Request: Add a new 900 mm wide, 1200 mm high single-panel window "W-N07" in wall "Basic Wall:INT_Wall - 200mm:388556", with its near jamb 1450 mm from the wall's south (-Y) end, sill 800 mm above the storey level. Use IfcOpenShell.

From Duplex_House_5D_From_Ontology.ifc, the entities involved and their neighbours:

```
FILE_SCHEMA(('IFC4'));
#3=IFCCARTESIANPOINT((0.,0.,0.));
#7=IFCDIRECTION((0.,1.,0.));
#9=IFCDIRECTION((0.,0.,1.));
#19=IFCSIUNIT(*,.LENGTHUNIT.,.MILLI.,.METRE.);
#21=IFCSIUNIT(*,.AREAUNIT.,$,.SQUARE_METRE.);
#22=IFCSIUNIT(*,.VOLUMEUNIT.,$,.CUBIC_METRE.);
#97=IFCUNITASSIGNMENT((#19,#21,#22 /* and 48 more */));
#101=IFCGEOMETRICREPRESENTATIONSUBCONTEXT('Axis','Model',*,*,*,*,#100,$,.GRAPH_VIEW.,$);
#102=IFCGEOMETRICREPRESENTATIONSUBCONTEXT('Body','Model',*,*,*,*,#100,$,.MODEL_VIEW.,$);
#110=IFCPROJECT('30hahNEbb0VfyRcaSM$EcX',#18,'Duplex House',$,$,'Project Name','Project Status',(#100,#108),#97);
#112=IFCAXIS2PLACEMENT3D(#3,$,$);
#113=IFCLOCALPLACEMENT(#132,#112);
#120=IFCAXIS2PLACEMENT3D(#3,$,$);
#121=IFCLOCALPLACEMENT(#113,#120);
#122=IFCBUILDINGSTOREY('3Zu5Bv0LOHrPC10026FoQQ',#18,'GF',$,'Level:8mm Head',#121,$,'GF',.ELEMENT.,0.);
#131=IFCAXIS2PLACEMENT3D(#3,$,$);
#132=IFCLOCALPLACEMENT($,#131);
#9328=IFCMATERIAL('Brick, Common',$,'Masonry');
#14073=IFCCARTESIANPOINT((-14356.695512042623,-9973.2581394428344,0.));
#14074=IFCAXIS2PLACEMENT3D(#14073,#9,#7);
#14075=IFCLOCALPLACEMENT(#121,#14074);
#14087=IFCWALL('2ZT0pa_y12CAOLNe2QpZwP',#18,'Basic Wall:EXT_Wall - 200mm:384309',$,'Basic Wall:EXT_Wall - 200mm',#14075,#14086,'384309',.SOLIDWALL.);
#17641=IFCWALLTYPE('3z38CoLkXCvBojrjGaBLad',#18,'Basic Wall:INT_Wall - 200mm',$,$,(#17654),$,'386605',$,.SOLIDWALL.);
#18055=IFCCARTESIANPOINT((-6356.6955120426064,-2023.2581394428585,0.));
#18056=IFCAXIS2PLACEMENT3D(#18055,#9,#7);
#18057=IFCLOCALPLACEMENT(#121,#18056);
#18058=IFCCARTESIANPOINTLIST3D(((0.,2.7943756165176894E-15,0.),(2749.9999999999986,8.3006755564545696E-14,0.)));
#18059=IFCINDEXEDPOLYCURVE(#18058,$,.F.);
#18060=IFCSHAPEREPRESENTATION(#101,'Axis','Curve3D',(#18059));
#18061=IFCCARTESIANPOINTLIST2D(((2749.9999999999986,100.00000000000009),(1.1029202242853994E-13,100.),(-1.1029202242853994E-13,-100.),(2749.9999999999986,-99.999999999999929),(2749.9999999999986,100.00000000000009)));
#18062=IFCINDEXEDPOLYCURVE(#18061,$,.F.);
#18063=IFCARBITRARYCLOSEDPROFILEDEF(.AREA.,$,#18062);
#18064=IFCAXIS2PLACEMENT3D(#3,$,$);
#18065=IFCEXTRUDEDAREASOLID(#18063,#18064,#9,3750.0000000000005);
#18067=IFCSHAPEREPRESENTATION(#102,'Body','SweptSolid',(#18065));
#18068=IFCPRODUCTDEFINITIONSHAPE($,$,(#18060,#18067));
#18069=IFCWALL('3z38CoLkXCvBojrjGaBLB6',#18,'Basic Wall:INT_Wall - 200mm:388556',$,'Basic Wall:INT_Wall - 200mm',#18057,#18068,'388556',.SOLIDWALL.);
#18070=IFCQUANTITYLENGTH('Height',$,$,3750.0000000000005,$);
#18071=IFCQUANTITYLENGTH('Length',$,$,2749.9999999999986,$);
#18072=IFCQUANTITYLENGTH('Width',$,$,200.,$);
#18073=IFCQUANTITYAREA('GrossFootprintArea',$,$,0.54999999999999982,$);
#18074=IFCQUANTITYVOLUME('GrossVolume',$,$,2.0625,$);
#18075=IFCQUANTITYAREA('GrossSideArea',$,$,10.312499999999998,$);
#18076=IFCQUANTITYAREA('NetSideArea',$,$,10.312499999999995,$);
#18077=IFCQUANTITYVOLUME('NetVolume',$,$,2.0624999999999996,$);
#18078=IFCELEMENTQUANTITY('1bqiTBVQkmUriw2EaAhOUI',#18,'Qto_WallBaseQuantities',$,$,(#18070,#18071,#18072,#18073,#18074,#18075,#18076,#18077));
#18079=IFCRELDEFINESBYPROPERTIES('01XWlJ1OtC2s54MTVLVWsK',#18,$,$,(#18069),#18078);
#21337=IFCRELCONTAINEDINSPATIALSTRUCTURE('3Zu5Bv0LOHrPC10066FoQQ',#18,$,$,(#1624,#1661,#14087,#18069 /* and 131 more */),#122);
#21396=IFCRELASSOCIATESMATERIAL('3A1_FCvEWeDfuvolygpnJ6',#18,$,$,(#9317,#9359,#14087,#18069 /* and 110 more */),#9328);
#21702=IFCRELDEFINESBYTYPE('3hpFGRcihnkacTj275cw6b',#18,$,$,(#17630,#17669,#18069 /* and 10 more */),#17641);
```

```python
import numpy as np
import ifcopenshell
import ifcopenshell.api.feature
import ifcopenshell.api.geometry
import ifcopenshell.api.pset
import ifcopenshell.api.root
import ifcopenshell.api.spatial
import ifcopenshell.geom
import ifcopenshell.util.element
import ifcopenshell.util.placement
import ifcopenshell.util.representation
import ifcopenshell.util.shape
import ifcopenshell.util.unit

model = ifcopenshell.open("Duplex_House_5D_From_Ontology.ifc")
unit_scale = ifcopenshell.util.unit.calculate_unit_scale(model)
area_scale = ifcopenshell.util.unit.calculate_unit_scale(model, "AREAUNIT")
volume_scale = ifcopenshell.util.unit.calculate_unit_scale(model, "VOLUMEUNIT")
settings = ifcopenshell.geom.settings()


def volume(element):
    """Net volume in cubic metres, openings subtracted."""
    shape = ifcopenshell.geom.create_shape(settings, element)
    return ifcopenshell.util.shape.get_volume(shape.geometry)


wall = model.by_guid("3z38CoLkXCvBojrjGaBLB6")
storey = ifcopenshell.util.element.get_container(wall, ifc_class="IfcBuildingStorey")
context = ifcopenshell.util.representation.get_context(model, "Model", "Body", "MODEL_VIEW")
before = volume(wall)

width, height, from_end, sill = 0.9, 1.2, 1.45, 0.8  # metres

# The wall runs along its own X axis, and the end named is its -X end.
wall_shape = ifcopenshell.geom.create_shape(settings, wall)
x, y, z = ifcopenshell.util.shape.get_vertices(wall_shape.geometry).T
start = x.min() + from_end
face, thickness = float(y.min()), float(y.max() - y.min())
wall_matrix = ifcopenshell.util.placement.get_local_placement(wall.ObjectPlacement)
level = ifcopenshell.util.placement.get_local_placement(storey.ObjectPlacement)[2, 3]


def in_wall(x, y):
    """Placement at x, y metres in the wall's axes, at sill height."""
    matrix = wall_matrix.copy()
    matrix[:, 3] = wall_matrix @ np.array([x / unit_scale, y / unit_scale, 0.0, 1.0])
    matrix[2, 3] = level + sill / unit_scale
    return matrix


# Opening: a box that overshoots both wall faces by 50 mm.
opening = ifcopenshell.api.root.create_entity(model, ifc_class="IfcOpeningElement", predefined_type="OPENING")
box = ifcopenshell.api.geometry.add_wall_representation(
    model, context=context, length=width, height=height, thickness=thickness + 0.1
)
ifcopenshell.api.geometry.assign_representation(model, product=opening, representation=box)
ifcopenshell.api.geometry.edit_object_placement(model, product=opening, matrix=in_wall(start, face - 0.05), is_si=False)
ifcopenshell.api.feature.add_feature(model, feature=opening, element=wall)

window = ifcopenshell.api.root.create_entity(model, ifc_class="IfcWindow", name="W-N07", predefined_type="WINDOW")
window.OverallWidth, window.OverallHeight = width / unit_scale, height / unit_scale
window.PartitioningType = "SINGLE_PANEL"
body = ifcopenshell.api.geometry.add_window_representation(
    model,
    context=context,
    overall_width=window.OverallWidth,
    overall_height=window.OverallHeight,
    partition_type="SINGLE_PANEL",
)
ifcopenshell.api.geometry.assign_representation(model, product=window, representation=body)
ifcopenshell.api.spatial.assign_container(model, products=[window], relating_structure=storey)
ifcopenshell.api.feature.add_filling(model, opening=opening, element=window)

# Centre the window in the wall's thickness.
ifcopenshell.api.geometry.edit_object_placement(model, product=window, matrix=in_wall(start, face), is_si=False)
window_shape = ifcopenshell.geom.create_shape(settings, window)
depth = ifcopenshell.util.shape.get_vertices(window_shape.geometry)[:, 1]
offset = face + thickness / 2 - (depth.min() + depth.max()) / 2
ifcopenshell.api.geometry.edit_object_placement(model, product=window, matrix=in_wall(start, offset), is_si=False)

after = volume(wall)

# Update the wall's stored quantities.
qto = model.by_id(ifcopenshell.util.element.get_pset(wall, "Qto_WallBaseQuantities", should_inherit=False)["id"])
ifcopenshell.api.pset.edit_qto(model, qto=qto, properties={
    "NetSideArea": after / thickness / area_scale,
    "NetVolume": after / volume_scale,
})

print(f"wall volume {before:.3f} -> {after:.3f} m3")

model.write("Duplex_House_5D_From_Ontology_edited.ifc")
```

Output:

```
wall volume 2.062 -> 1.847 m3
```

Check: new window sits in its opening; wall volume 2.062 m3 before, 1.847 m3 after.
